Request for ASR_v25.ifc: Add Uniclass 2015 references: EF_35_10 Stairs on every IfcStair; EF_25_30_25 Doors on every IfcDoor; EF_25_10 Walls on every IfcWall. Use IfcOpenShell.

First a look at what the model holds.

```python
import ifcopenshell

model = ifcopenshell.open("ASR_v25.ifc")
print(model.schema)
print("classifications:", [c.Name for c in model.by_type("IfcClassification")])
for ifc_class in ("IfcDoor", "IfcRoof", "IfcStair", "IfcWall", "IfcWindow"):
    print(ifc_class, len(model.by_type(ifc_class)))
```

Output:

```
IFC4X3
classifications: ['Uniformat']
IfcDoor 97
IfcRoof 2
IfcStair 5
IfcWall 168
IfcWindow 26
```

```python
import ifcopenshell
import ifcopenshell.api.classification

model = ifcopenshell.open("ASR_v25.ifc")

system = ifcopenshell.api.classification.add_classification(model, classification="Uniclass 2015")

codes = {
    "IfcStair": ("EF_35_10", "Stairs"),
    "IfcDoor": ("EF_25_30_25", "Doors"),
    "IfcWall": ("EF_25_10", "Walls"),
}
for ifc_class, (code, name) in codes.items():
    products = model.by_type(ifc_class)
    ifcopenshell.api.classification.add_reference(
        model, products=products, classification=system, identification=code, name=name
    )
    print(code, len(products))

model.write("ASR_v25_edited.ifc")
```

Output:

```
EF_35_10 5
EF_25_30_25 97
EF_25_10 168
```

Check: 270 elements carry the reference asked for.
